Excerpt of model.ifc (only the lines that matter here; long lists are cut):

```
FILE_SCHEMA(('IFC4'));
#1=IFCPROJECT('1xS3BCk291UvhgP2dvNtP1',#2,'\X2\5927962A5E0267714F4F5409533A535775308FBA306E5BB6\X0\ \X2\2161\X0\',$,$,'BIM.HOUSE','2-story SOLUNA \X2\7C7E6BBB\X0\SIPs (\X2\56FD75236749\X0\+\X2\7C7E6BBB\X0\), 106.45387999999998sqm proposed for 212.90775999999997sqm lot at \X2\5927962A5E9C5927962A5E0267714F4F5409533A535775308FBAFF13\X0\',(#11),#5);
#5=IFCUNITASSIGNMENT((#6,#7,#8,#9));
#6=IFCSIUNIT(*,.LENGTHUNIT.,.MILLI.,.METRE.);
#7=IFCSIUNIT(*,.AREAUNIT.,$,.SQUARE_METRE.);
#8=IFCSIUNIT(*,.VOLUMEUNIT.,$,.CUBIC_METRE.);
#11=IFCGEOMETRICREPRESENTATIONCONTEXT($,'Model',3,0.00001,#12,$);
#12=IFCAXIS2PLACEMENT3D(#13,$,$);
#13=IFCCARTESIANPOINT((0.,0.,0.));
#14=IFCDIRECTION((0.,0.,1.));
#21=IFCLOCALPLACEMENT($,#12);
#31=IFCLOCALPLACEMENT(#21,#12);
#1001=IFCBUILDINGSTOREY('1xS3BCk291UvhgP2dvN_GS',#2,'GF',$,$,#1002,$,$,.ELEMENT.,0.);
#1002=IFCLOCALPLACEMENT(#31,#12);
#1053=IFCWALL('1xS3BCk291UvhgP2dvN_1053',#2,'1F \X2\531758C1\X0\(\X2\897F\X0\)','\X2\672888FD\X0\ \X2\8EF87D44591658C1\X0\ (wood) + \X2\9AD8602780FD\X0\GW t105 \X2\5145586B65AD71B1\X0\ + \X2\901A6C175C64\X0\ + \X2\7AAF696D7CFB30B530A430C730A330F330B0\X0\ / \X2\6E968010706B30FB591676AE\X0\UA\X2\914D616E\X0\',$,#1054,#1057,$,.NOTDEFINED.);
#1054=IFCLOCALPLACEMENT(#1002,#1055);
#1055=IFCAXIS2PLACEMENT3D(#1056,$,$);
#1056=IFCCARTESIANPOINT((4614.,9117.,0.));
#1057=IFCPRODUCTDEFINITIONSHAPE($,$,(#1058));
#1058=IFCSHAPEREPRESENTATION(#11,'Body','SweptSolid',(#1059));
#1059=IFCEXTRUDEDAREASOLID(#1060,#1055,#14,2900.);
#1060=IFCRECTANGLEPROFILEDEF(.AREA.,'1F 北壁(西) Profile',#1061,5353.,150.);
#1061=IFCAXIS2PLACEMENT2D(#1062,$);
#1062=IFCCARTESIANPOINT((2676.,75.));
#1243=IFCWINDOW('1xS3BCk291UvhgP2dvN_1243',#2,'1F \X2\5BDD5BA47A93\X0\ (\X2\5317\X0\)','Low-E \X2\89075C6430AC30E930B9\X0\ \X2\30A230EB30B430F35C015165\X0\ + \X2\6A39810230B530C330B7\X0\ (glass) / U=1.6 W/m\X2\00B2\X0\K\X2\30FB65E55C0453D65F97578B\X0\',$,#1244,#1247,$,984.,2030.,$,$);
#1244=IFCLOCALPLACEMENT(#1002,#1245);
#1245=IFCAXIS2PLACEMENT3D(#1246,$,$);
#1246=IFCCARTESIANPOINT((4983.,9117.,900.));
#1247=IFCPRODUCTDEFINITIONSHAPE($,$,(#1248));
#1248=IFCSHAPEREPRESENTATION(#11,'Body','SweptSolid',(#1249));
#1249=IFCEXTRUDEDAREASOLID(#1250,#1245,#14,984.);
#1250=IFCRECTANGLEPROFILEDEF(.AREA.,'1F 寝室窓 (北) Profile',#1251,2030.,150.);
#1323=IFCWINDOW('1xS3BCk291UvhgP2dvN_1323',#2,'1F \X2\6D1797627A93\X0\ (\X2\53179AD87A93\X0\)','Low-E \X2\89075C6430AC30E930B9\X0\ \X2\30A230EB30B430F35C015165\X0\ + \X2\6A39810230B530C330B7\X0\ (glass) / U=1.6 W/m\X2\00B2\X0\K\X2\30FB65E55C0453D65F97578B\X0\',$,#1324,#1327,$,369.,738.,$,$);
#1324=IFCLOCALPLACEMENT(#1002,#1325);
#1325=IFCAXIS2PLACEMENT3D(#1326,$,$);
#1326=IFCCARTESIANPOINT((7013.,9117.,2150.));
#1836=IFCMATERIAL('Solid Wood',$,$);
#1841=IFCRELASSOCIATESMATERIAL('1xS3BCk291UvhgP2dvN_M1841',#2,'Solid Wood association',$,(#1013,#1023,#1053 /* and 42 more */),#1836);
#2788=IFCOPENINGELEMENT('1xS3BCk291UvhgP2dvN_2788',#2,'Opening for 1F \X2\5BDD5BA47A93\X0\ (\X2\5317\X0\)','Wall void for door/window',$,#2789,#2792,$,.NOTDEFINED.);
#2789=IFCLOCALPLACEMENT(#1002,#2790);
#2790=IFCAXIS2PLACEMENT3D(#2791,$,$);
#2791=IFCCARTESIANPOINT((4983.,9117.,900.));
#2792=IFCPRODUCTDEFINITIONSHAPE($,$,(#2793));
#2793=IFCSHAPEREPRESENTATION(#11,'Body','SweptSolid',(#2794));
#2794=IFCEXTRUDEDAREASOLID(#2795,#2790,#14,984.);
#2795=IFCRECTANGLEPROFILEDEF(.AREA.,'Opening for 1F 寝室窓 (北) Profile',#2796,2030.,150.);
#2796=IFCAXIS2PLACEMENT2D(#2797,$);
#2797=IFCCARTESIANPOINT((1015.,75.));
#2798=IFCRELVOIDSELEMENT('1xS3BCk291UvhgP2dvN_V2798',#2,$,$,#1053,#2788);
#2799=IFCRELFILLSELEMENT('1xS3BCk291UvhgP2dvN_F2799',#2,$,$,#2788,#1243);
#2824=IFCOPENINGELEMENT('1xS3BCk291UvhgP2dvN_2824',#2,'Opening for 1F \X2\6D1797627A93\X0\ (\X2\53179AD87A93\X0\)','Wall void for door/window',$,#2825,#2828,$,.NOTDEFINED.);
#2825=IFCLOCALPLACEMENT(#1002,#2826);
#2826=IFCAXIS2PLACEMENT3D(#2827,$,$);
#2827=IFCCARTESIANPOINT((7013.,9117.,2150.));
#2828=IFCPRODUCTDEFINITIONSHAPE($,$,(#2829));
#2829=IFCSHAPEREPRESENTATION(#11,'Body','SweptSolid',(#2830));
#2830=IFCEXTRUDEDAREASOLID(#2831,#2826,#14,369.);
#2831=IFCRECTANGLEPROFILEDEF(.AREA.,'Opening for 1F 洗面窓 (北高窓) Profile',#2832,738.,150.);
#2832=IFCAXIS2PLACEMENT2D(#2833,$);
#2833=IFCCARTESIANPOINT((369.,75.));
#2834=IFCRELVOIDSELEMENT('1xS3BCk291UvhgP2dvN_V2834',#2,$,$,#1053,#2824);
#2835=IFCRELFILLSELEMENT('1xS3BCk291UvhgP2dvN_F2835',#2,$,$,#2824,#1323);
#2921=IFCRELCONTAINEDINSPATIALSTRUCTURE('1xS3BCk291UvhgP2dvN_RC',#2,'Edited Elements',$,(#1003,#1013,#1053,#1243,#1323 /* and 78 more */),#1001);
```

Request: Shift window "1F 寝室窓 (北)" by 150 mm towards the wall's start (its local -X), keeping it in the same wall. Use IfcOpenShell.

```python
import ifcopenshell
import ifcopenshell.api.geometry
import ifcopenshell.util.placement
import ifcopenshell.util.unit

model = ifcopenshell.open("model.ifc")
unit_scale = ifcopenshell.util.unit.calculate_unit_scale(model)

window = model.by_id(1243)
opening = window.FillsVoids[0].RelatingOpeningElement
wall = opening.VoidsElements[0].RelatingBuildingElement

wall_matrix = ifcopenshell.util.placement.get_local_placement(wall.ObjectPlacement)
shift = wall_matrix[:3, 0] * -0.15 / unit_scale
before = ifcopenshell.util.placement.get_local_placement(window.ObjectPlacement)[:3, 3].copy()

# The window is not placed relative to its opening, so move both.
for product in (opening, window):
    matrix = ifcopenshell.util.placement.get_local_placement(product.ObjectPlacement)
    matrix[:3, 3] += shift
    ifcopenshell.api.geometry.edit_object_placement(model, product=product, matrix=matrix, is_si=False)

after = ifcopenshell.util.placement.get_local_placement(window.ObjectPlacement)[:3, 3]
print("window moved by", (after - before).round(3) + 0.0)

model.write("model_v2.ifc")
```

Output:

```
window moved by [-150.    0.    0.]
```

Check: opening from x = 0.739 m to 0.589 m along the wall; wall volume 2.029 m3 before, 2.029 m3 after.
